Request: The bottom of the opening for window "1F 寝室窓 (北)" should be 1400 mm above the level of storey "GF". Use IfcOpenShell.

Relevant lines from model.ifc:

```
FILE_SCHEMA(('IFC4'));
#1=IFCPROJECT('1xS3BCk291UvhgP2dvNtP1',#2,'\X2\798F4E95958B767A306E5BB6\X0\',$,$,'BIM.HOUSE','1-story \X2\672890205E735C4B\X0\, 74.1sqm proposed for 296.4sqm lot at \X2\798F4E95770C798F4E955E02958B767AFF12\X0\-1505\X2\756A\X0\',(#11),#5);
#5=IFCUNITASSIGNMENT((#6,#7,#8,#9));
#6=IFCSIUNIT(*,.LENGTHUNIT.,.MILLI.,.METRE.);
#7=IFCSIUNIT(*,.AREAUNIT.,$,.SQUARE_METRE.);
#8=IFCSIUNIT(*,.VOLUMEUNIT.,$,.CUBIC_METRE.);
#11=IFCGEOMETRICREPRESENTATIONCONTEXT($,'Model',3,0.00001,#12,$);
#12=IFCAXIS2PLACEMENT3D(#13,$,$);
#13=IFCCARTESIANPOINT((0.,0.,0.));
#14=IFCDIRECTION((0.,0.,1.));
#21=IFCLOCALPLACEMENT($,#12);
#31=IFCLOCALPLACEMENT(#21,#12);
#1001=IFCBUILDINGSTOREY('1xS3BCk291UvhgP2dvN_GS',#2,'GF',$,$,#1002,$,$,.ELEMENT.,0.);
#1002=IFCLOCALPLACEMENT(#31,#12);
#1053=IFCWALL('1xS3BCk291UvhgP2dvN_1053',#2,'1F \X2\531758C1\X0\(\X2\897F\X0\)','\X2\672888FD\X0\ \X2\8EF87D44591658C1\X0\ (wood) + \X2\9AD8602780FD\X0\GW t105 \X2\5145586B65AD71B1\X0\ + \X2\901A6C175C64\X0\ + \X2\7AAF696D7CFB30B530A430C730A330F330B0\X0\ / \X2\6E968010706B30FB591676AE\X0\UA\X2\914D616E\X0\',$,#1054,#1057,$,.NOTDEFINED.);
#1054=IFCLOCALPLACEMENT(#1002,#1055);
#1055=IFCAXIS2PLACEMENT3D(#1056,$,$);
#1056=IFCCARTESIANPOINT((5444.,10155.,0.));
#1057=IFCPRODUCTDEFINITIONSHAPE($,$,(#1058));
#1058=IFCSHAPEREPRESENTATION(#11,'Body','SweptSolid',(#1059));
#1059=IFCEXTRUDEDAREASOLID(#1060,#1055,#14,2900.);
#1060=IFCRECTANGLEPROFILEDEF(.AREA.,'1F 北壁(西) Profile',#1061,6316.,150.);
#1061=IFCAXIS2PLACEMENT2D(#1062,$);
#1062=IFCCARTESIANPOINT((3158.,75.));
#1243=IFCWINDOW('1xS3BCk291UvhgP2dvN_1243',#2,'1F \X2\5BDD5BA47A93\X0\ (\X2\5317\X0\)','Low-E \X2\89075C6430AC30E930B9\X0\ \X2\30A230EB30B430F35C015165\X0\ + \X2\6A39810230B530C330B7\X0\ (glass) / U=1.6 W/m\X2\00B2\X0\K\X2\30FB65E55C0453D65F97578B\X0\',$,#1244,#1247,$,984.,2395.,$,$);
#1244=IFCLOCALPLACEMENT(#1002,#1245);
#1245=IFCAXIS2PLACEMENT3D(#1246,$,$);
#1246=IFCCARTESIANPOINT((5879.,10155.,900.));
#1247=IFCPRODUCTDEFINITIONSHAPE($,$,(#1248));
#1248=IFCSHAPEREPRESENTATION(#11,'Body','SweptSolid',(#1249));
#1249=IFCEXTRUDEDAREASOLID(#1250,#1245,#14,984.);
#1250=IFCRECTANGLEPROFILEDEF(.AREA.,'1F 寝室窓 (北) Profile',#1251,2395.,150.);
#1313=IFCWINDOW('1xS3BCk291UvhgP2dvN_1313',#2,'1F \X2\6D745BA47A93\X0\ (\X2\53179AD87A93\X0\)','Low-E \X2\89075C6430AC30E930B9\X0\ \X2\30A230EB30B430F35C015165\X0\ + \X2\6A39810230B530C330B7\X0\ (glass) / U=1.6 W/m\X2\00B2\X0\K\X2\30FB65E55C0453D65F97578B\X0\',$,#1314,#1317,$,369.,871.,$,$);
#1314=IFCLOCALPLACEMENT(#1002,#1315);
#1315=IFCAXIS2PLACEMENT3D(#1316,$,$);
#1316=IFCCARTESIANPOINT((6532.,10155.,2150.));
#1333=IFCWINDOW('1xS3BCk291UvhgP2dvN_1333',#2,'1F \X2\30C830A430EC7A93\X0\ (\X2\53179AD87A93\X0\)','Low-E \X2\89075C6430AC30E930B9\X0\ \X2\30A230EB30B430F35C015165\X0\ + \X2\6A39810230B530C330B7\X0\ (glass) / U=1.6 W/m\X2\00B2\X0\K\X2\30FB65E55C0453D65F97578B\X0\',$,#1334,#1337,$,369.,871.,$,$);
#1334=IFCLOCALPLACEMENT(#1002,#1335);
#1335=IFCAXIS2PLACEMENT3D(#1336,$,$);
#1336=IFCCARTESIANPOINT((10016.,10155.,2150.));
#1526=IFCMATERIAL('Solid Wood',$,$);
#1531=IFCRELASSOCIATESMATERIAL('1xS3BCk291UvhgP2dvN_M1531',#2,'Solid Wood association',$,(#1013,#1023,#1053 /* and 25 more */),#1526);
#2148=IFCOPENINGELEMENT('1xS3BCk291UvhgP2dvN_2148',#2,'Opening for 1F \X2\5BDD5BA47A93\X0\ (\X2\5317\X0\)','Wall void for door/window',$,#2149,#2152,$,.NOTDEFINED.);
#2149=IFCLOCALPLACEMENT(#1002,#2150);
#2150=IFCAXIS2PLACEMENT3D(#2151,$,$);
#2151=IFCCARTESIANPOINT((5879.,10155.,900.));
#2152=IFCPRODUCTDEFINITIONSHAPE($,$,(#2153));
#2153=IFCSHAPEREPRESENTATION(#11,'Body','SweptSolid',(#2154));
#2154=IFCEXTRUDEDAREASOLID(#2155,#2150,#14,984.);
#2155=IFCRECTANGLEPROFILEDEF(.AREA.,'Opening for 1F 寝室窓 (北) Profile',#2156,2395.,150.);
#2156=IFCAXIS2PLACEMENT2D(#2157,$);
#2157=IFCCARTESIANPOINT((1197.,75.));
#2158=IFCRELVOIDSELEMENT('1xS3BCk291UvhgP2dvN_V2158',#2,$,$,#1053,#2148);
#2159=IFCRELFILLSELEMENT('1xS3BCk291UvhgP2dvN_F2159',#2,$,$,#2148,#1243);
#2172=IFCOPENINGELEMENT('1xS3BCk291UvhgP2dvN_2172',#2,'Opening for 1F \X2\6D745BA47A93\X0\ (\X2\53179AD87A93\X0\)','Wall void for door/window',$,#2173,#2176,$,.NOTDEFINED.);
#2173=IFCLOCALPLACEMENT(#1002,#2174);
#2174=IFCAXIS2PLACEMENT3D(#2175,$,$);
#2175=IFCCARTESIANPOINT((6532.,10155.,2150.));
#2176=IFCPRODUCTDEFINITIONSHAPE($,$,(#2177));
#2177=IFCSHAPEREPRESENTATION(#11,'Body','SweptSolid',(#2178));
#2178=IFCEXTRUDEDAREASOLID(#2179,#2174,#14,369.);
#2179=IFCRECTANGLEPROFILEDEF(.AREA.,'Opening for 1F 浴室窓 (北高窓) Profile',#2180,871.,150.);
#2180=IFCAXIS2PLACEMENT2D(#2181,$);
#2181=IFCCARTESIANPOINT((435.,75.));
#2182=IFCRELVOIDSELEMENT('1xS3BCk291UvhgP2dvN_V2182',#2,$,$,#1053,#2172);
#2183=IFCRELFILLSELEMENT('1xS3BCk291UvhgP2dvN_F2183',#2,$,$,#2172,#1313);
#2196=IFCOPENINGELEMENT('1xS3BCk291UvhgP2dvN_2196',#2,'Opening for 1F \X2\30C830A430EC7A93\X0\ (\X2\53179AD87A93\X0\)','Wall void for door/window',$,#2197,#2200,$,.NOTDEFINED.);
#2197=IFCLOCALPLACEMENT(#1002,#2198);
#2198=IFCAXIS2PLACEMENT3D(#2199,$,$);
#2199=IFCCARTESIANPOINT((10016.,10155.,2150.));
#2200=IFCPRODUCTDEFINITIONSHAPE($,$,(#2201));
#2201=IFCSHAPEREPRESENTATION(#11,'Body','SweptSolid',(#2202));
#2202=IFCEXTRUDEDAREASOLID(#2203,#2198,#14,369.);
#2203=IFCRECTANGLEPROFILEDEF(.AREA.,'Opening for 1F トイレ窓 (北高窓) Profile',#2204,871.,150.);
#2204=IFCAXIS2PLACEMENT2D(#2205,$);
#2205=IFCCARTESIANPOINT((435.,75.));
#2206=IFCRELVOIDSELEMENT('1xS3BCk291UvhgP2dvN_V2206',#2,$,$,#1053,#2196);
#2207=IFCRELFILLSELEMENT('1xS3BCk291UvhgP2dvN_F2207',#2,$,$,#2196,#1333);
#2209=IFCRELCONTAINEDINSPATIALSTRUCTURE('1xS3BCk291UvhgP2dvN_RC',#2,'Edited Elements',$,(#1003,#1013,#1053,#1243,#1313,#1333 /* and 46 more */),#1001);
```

```python
import numpy as np
import ifcopenshell
import ifcopenshell.api.geometry
import ifcopenshell.geom
import ifcopenshell.util.element
import ifcopenshell.util.placement
import ifcopenshell.util.shape
import ifcopenshell.util.unit

model = ifcopenshell.open("model.ifc")
unit_scale = ifcopenshell.util.unit.calculate_unit_scale(model)

window = model.by_id(1243)
opening = window.FillsVoids[0].RelatingOpeningElement
storey = ifcopenshell.util.element.get_container(window, ifc_class="IfcBuildingStorey")
level = ifcopenshell.util.placement.get_local_placement(storey.ObjectPlacement)[2, 3]

# The opening's origin need not be at the sill, so measure its lowest point.
shape = ifcopenshell.geom.create_shape(ifcopenshell.geom.settings(), opening)
bottom = ifcopenshell.util.shape.get_shape_bottom_elevation(shape, shape.geometry) / unit_scale
dz = level + 1400.0 - bottom

shift = np.array([0.0, 0.0, dz])
# The window is not placed relative to its opening, so move both.
for product in (opening, window):
    matrix = ifcopenshell.util.placement.get_local_placement(product.ObjectPlacement)
    matrix[:3, 3] += shift
    ifcopenshell.api.geometry.edit_object_placement(model, product=product, matrix=matrix, is_si=False)

print(f"moved by {dz * unit_scale:+.3f} m")

model.write("model-out.ifc")
```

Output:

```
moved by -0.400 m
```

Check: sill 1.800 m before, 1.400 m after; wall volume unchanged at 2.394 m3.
